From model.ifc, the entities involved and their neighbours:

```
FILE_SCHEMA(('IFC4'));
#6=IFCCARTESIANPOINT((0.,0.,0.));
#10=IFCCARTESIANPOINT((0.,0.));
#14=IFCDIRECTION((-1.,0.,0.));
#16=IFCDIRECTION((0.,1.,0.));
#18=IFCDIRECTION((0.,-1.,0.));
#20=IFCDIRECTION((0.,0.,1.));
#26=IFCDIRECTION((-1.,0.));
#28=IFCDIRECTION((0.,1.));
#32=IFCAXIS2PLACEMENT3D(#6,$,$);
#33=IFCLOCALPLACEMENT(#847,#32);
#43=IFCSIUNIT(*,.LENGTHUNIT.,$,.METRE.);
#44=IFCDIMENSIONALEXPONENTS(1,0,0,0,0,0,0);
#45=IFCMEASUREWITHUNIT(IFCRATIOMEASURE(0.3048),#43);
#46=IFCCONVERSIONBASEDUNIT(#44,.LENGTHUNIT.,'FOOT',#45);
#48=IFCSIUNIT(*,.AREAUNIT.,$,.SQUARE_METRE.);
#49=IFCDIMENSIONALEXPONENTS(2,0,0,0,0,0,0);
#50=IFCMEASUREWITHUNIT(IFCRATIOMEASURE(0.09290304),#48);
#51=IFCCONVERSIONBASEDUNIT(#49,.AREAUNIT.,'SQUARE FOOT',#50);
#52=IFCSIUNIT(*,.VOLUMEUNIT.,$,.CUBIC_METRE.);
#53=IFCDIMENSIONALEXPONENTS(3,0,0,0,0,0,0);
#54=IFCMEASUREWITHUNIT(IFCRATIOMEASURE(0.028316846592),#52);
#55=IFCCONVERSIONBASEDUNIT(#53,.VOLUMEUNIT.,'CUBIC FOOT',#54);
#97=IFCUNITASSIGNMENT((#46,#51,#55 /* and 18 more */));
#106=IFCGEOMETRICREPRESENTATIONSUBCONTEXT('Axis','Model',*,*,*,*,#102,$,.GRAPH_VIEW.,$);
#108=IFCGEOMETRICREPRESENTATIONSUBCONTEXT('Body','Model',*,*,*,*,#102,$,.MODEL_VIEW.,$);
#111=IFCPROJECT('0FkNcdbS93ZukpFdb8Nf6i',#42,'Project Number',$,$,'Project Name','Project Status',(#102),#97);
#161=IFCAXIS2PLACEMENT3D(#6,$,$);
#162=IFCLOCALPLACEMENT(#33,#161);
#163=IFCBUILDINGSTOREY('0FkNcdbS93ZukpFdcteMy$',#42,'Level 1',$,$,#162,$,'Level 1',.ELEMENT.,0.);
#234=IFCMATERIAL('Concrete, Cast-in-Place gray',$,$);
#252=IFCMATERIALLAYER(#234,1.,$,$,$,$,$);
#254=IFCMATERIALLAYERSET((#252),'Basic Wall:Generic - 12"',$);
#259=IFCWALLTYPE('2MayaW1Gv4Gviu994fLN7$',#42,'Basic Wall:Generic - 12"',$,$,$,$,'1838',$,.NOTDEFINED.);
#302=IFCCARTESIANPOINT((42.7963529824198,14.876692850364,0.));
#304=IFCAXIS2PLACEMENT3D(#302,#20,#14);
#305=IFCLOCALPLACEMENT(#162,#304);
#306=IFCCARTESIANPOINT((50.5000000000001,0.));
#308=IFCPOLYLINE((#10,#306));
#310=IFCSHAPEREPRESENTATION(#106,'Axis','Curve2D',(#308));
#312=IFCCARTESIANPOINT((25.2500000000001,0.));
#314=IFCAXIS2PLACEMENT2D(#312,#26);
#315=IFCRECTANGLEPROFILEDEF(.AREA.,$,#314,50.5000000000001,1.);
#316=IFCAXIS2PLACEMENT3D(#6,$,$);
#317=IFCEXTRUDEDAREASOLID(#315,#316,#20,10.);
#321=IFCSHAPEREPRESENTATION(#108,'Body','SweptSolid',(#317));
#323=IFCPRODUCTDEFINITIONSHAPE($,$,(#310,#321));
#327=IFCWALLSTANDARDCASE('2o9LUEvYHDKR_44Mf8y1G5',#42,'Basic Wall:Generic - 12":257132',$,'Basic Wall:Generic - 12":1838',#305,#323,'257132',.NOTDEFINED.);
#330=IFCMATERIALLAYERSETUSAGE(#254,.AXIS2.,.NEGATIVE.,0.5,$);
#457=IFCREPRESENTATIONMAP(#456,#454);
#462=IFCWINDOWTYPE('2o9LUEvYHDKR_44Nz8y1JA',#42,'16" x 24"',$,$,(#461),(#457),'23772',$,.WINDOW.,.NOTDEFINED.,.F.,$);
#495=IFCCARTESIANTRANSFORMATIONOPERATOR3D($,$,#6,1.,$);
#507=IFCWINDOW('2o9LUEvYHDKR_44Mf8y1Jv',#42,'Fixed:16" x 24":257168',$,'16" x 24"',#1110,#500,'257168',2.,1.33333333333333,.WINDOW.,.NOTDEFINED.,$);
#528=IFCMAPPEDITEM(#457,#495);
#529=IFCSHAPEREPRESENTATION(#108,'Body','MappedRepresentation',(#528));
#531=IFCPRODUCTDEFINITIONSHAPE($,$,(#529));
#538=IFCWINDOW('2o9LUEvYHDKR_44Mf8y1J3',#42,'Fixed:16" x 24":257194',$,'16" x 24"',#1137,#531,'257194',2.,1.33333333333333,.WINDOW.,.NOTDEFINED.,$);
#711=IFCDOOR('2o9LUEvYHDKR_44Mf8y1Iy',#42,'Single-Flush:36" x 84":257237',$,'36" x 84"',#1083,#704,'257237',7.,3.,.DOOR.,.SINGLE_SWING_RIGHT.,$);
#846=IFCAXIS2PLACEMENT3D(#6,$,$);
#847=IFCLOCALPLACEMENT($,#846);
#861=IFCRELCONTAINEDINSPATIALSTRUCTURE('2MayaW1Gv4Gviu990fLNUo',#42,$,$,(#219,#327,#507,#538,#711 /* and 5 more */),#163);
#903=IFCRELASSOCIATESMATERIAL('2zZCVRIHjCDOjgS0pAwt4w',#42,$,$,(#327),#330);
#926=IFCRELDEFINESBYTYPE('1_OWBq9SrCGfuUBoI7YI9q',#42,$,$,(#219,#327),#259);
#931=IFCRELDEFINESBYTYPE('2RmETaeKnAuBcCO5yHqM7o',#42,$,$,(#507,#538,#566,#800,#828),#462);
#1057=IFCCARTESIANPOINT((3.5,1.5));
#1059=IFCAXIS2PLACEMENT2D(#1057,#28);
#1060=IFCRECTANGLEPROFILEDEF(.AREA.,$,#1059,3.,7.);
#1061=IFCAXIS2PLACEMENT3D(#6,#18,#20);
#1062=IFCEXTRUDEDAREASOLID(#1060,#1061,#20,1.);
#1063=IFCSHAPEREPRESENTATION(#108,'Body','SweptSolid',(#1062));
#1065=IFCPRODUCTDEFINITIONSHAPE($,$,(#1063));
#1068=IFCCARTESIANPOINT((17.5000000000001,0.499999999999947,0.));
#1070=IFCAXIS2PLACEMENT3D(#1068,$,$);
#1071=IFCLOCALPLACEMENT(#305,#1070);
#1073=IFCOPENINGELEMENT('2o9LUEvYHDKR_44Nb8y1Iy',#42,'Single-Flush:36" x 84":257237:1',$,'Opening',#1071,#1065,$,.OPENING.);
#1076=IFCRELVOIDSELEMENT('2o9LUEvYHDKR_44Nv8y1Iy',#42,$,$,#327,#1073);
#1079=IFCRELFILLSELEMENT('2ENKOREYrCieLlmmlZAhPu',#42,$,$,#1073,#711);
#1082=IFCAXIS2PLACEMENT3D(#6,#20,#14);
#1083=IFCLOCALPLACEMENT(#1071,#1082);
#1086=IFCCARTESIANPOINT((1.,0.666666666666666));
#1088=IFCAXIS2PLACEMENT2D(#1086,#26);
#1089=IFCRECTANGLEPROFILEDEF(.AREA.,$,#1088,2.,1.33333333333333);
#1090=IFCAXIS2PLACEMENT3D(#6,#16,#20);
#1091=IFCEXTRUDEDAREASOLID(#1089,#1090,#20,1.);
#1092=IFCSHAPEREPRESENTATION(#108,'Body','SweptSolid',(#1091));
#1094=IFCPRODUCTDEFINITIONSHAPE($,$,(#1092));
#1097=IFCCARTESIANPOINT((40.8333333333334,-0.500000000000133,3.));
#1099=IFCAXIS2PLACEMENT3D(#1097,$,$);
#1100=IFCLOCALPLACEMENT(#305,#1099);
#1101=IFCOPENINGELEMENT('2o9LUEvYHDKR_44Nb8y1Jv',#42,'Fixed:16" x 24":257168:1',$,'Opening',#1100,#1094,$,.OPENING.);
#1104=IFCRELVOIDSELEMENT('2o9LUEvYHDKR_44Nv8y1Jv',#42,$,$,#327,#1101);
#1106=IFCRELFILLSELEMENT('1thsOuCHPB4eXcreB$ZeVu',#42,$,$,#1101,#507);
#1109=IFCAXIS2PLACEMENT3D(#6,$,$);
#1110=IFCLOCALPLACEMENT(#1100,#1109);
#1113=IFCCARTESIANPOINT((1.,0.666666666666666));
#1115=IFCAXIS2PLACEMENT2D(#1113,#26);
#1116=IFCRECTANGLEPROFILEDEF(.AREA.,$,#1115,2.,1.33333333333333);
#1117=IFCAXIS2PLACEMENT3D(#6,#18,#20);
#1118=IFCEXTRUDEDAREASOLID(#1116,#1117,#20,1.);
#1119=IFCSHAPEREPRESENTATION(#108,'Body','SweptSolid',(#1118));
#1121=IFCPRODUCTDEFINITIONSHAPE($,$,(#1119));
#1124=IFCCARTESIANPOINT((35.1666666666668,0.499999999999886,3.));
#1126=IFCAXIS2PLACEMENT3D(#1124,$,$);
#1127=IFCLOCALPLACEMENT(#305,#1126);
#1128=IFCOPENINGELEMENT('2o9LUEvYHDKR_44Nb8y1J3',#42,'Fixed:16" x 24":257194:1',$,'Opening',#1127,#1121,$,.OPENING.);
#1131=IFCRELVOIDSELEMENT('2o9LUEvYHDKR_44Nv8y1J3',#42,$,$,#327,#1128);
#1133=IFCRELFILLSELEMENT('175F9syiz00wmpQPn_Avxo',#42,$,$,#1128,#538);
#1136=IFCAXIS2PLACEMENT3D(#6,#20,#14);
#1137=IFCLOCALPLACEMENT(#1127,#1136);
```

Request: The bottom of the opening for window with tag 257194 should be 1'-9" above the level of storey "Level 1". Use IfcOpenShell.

```python
import numpy as np
import ifcopenshell
import ifcopenshell.api.geometry
import ifcopenshell.geom
import ifcopenshell.util.element
import ifcopenshell.util.placement
import ifcopenshell.util.shape
import ifcopenshell.util.unit

model = ifcopenshell.open("model.ifc")
unit_scale = ifcopenshell.util.unit.calculate_unit_scale(model)

window = model.by_guid("2o9LUEvYHDKR_44Mf8y1J3")
opening = window.FillsVoids[0].RelatingOpeningElement
storey = ifcopenshell.util.element.get_container(window, ifc_class="IfcBuildingStorey")
level = ifcopenshell.util.placement.get_local_placement(storey.ObjectPlacement)[2, 3]

# The opening's origin need not be at the sill, so measure its lowest point.
shape = ifcopenshell.geom.create_shape(ifcopenshell.geom.settings(), opening)
bottom = ifcopenshell.util.shape.get_shape_bottom_elevation(shape, shape.geometry) / unit_scale
dz = level + 21 * 0.0254 / unit_scale - bottom

shift = np.array([0.0, 0.0, dz])
# The window is placed relative to its opening, so it follows when the opening moves.
matrix = ifcopenshell.util.placement.get_local_placement(opening.ObjectPlacement)
matrix[:3, 3] += shift
ifcopenshell.api.geometry.edit_object_placement(
    model, product=opening, matrix=matrix, is_si=False, should_transform_children=True
)

print(f"moved by {dz * unit_scale:+.3f} m")

model.write("model_updated.ifc")
```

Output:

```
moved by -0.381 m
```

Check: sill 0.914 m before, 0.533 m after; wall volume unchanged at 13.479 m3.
